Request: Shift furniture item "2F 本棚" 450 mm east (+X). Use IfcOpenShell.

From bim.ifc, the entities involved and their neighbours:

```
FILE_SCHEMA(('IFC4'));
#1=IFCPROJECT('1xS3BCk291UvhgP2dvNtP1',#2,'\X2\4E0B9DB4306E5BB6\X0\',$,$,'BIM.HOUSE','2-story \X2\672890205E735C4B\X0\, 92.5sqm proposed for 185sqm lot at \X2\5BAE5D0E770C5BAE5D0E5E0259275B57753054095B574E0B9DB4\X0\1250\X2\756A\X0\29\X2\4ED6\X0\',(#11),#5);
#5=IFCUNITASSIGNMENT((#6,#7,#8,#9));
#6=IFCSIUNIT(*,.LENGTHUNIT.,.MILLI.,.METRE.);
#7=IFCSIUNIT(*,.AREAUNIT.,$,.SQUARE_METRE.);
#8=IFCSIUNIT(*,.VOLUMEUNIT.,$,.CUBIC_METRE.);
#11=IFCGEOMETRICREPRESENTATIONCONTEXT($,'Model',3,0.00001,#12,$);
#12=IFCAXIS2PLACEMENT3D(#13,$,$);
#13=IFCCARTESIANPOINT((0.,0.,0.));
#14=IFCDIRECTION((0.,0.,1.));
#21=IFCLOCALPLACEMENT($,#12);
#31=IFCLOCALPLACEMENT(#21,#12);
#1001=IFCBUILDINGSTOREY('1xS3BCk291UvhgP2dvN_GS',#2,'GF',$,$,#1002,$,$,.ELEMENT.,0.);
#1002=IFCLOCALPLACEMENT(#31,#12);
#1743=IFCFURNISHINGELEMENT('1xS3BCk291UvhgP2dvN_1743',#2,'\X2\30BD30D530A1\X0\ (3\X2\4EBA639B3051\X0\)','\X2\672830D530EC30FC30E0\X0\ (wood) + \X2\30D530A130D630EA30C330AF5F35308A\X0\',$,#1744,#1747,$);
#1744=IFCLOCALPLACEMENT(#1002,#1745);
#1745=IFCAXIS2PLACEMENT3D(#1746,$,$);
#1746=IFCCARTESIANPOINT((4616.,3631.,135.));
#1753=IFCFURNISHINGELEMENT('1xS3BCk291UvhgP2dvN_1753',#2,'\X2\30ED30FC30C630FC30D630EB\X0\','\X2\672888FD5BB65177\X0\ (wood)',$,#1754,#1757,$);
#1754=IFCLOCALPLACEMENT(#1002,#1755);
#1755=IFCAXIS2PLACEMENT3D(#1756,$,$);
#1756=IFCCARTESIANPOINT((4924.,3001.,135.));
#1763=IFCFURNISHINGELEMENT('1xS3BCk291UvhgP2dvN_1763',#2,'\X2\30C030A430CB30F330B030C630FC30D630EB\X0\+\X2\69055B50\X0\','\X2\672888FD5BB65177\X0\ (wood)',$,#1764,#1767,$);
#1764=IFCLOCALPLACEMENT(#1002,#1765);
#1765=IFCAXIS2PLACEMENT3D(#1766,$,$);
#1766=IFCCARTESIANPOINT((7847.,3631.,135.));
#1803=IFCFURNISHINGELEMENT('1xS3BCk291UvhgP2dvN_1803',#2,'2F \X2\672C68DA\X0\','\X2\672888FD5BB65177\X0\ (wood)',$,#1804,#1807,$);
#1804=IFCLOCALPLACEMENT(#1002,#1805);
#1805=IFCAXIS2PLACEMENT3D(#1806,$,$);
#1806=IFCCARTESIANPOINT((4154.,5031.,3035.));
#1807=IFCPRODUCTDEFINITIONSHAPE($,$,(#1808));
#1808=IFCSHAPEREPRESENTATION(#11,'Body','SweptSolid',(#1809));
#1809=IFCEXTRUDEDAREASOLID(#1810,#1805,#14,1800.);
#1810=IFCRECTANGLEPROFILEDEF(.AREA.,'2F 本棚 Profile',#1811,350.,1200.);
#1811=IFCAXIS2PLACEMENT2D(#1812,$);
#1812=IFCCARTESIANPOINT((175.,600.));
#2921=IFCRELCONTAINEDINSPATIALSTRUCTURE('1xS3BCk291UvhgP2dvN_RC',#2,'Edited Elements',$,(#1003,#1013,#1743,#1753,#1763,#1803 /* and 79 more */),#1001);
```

```python
import ifcopenshell
import ifcopenshell.api.geometry
import ifcopenshell.util.placement
import ifcopenshell.util.unit

model = ifcopenshell.open("bim.ifc")
unit_scale = ifcopenshell.util.unit.calculate_unit_scale(model)

item = model.by_guid("1xS3BCk291UvhgP2dvN_1803")
matrix = ifcopenshell.util.placement.get_local_placement(item.ObjectPlacement)
matrix[0, 3] += 0.45 / unit_scale
ifcopenshell.api.geometry.edit_object_placement(model, product=item, matrix=matrix, is_si=False)

print(ifcopenshell.util.placement.get_local_placement(item.ObjectPlacement).round(3) + 0.0)

model.write("bim_updated.ifc")
```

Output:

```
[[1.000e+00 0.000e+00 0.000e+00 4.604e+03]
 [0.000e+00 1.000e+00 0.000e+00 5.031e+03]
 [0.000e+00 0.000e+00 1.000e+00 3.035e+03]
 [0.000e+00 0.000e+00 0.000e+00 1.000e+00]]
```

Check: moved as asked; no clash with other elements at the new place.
